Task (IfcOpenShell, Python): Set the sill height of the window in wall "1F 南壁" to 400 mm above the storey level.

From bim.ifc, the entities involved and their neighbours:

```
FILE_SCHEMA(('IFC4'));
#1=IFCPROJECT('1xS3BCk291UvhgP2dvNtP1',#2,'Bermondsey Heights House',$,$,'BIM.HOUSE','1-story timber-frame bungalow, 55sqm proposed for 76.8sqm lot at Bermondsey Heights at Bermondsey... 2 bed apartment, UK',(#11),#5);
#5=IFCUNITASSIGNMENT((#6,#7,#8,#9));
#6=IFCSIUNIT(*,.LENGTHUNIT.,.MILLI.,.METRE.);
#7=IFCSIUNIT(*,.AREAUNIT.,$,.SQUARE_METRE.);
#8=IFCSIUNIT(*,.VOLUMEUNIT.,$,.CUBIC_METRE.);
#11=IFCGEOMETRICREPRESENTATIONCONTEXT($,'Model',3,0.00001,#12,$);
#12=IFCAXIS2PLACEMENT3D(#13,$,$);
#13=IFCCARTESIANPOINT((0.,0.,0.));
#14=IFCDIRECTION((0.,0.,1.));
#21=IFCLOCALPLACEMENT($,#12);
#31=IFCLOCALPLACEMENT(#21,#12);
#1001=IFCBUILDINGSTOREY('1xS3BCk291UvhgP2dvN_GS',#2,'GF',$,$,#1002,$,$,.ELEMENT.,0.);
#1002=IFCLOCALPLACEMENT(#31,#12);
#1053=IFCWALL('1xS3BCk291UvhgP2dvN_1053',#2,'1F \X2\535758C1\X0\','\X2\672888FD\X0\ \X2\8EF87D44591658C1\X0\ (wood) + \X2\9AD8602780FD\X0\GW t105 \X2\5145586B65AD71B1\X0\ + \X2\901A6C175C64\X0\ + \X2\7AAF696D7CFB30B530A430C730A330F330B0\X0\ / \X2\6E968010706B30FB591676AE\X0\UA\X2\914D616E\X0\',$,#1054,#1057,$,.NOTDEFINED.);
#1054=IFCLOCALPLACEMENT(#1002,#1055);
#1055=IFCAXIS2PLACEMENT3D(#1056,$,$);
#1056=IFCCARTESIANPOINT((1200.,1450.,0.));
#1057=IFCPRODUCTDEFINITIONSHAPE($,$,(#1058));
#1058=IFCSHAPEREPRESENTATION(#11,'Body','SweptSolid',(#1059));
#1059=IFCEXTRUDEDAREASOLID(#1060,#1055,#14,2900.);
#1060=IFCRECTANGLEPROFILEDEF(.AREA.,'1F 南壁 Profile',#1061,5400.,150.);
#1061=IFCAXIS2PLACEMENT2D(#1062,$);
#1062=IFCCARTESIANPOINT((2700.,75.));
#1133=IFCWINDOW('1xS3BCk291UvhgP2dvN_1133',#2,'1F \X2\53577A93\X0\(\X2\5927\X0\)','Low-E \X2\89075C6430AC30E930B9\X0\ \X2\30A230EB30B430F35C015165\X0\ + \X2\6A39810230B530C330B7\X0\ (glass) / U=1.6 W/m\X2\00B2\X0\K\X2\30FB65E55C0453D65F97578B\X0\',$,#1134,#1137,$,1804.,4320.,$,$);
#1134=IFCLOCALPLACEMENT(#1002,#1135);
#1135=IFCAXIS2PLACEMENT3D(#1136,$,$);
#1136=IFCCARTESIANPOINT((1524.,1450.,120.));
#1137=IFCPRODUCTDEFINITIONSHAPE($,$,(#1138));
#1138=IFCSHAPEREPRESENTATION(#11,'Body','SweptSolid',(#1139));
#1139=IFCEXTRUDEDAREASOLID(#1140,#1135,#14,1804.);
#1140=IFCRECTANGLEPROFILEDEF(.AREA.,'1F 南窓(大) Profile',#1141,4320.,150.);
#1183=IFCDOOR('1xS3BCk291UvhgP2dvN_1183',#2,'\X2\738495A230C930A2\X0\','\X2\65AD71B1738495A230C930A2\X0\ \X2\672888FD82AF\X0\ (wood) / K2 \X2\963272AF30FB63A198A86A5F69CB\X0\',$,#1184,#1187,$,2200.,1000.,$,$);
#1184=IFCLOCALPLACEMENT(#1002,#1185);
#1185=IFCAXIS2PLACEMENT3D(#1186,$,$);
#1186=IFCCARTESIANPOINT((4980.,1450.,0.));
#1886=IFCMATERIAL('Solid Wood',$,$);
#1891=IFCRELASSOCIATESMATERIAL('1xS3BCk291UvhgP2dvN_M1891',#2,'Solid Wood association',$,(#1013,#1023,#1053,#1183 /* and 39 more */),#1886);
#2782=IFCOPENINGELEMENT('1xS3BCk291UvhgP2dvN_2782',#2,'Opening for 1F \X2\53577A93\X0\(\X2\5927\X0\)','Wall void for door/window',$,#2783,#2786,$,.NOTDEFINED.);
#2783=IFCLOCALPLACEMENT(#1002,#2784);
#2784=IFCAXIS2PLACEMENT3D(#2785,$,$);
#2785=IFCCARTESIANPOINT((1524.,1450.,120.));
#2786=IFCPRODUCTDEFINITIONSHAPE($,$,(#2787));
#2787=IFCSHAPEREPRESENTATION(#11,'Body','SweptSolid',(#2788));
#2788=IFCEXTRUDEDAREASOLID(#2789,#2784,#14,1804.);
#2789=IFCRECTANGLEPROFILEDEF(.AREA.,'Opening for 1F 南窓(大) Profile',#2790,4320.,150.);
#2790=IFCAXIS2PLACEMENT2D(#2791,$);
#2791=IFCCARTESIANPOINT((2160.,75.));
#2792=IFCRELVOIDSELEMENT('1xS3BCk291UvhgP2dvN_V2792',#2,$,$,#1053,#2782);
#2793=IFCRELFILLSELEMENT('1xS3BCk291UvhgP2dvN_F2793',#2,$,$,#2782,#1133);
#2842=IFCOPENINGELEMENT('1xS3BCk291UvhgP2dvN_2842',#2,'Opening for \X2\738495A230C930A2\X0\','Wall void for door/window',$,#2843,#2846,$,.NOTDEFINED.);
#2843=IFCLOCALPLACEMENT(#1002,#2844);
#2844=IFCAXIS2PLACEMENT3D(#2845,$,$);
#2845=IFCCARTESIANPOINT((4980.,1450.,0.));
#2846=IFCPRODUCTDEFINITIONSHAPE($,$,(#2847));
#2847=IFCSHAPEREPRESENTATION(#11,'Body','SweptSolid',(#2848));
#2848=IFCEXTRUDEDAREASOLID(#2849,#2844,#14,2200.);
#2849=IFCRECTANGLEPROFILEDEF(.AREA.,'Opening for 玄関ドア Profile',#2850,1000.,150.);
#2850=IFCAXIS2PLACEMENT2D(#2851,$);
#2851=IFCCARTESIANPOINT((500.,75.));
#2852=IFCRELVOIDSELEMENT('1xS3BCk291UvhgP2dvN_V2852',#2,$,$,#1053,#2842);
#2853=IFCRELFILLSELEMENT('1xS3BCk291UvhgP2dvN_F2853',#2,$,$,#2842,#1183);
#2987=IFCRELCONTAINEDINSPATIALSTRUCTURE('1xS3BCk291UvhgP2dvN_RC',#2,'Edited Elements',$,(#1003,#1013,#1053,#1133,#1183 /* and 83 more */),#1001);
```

```python
import numpy as np
import ifcopenshell
import ifcopenshell.api.geometry
import ifcopenshell.geom
import ifcopenshell.util.element
import ifcopenshell.util.placement
import ifcopenshell.util.shape
import ifcopenshell.util.unit

model = ifcopenshell.open("bim.ifc")
unit_scale = ifcopenshell.util.unit.calculate_unit_scale(model)

window = model.by_guid("1xS3BCk291UvhgP2dvN_1133")
opening = window.FillsVoids[0].RelatingOpeningElement
storey = ifcopenshell.util.element.get_container(window, ifc_class="IfcBuildingStorey")
level = ifcopenshell.util.placement.get_local_placement(storey.ObjectPlacement)[2, 3]

# The opening's origin need not be at the sill, so measure its lowest point.
shape = ifcopenshell.geom.create_shape(ifcopenshell.geom.settings(), opening)
bottom = ifcopenshell.util.shape.get_shape_bottom_elevation(shape, shape.geometry) / unit_scale
dz = level + 400.0 - bottom

shift = np.array([0.0, 0.0, dz])
# The window is not placed relative to its opening, so move both.
for product in (opening, window):
    matrix = ifcopenshell.util.placement.get_local_placement(product.ObjectPlacement)
    matrix[:3, 3] += shift
    ifcopenshell.api.geometry.edit_object_placement(model, product=product, matrix=matrix, is_si=False)

print(f"moved by {dz * unit_scale:+.3f} m")

model.write("bim_rev.ifc")
```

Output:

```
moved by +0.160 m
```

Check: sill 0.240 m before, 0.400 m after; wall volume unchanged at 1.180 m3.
